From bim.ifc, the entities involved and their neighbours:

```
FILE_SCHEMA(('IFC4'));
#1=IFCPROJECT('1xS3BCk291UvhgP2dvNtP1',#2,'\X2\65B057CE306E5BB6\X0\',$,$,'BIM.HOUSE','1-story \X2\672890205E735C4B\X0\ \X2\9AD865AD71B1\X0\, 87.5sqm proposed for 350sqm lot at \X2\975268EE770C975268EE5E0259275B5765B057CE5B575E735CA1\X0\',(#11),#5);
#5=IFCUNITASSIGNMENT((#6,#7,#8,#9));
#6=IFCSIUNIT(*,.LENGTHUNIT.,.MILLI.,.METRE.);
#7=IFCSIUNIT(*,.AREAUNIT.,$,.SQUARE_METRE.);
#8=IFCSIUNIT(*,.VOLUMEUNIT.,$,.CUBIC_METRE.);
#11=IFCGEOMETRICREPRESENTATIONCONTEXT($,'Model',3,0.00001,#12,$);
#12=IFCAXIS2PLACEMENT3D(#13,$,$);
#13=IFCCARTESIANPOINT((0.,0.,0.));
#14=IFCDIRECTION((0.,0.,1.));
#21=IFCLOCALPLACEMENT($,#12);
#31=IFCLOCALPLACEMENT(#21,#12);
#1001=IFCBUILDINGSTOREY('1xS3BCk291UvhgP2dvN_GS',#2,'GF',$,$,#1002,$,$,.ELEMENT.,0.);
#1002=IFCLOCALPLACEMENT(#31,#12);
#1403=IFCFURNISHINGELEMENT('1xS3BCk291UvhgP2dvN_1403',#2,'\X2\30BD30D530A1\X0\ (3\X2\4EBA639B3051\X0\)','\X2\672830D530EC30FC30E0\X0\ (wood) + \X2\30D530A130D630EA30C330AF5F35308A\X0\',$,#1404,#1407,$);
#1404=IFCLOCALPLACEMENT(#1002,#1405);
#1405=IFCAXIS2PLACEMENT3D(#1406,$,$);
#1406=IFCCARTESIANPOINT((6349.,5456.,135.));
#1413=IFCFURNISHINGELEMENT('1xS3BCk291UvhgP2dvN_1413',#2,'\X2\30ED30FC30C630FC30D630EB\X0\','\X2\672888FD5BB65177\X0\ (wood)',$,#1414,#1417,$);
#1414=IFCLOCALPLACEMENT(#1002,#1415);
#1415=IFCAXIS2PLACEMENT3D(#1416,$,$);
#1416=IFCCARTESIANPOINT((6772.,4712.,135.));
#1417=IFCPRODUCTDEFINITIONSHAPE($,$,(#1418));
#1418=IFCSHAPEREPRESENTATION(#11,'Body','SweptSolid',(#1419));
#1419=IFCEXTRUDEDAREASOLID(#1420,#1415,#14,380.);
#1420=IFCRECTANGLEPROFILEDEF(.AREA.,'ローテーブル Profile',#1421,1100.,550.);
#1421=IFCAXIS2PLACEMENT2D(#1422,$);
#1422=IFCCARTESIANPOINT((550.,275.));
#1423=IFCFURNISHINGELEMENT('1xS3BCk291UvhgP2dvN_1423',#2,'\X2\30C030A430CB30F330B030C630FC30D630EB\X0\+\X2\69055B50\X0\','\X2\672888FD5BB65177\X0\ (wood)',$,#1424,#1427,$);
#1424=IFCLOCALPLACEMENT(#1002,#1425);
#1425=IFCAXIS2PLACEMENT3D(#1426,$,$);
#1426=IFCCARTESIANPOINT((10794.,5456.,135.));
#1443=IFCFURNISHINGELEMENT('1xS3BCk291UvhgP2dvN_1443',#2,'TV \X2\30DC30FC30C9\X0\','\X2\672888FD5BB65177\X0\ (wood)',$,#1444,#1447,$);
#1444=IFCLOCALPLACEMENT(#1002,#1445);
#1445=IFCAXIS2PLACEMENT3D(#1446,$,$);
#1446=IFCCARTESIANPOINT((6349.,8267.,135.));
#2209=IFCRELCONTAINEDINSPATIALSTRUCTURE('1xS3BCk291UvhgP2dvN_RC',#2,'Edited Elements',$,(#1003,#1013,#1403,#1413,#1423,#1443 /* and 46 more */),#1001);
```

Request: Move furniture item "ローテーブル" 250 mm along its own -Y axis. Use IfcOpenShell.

```python
import ifcopenshell
import ifcopenshell.api.geometry
import ifcopenshell.util.placement
import ifcopenshell.util.unit

model = ifcopenshell.open("bim.ifc")
unit_scale = ifcopenshell.util.unit.calculate_unit_scale(model)

item = model.by_guid("1xS3BCk291UvhgP2dvN_1413")
matrix = ifcopenshell.util.placement.get_local_placement(item.ObjectPlacement)
matrix[:3, 3] -= matrix[:3, 1] * 0.25 / unit_scale
ifcopenshell.api.geometry.edit_object_placement(model, product=item, matrix=matrix, is_si=False)

print(ifcopenshell.util.placement.get_local_placement(item.ObjectPlacement).round(3) + 0.0)

model.write("bim_rev.ifc")
```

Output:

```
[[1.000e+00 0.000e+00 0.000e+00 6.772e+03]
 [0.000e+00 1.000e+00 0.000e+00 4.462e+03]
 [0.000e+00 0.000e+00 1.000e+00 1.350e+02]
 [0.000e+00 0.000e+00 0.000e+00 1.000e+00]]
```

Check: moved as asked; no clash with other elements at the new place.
